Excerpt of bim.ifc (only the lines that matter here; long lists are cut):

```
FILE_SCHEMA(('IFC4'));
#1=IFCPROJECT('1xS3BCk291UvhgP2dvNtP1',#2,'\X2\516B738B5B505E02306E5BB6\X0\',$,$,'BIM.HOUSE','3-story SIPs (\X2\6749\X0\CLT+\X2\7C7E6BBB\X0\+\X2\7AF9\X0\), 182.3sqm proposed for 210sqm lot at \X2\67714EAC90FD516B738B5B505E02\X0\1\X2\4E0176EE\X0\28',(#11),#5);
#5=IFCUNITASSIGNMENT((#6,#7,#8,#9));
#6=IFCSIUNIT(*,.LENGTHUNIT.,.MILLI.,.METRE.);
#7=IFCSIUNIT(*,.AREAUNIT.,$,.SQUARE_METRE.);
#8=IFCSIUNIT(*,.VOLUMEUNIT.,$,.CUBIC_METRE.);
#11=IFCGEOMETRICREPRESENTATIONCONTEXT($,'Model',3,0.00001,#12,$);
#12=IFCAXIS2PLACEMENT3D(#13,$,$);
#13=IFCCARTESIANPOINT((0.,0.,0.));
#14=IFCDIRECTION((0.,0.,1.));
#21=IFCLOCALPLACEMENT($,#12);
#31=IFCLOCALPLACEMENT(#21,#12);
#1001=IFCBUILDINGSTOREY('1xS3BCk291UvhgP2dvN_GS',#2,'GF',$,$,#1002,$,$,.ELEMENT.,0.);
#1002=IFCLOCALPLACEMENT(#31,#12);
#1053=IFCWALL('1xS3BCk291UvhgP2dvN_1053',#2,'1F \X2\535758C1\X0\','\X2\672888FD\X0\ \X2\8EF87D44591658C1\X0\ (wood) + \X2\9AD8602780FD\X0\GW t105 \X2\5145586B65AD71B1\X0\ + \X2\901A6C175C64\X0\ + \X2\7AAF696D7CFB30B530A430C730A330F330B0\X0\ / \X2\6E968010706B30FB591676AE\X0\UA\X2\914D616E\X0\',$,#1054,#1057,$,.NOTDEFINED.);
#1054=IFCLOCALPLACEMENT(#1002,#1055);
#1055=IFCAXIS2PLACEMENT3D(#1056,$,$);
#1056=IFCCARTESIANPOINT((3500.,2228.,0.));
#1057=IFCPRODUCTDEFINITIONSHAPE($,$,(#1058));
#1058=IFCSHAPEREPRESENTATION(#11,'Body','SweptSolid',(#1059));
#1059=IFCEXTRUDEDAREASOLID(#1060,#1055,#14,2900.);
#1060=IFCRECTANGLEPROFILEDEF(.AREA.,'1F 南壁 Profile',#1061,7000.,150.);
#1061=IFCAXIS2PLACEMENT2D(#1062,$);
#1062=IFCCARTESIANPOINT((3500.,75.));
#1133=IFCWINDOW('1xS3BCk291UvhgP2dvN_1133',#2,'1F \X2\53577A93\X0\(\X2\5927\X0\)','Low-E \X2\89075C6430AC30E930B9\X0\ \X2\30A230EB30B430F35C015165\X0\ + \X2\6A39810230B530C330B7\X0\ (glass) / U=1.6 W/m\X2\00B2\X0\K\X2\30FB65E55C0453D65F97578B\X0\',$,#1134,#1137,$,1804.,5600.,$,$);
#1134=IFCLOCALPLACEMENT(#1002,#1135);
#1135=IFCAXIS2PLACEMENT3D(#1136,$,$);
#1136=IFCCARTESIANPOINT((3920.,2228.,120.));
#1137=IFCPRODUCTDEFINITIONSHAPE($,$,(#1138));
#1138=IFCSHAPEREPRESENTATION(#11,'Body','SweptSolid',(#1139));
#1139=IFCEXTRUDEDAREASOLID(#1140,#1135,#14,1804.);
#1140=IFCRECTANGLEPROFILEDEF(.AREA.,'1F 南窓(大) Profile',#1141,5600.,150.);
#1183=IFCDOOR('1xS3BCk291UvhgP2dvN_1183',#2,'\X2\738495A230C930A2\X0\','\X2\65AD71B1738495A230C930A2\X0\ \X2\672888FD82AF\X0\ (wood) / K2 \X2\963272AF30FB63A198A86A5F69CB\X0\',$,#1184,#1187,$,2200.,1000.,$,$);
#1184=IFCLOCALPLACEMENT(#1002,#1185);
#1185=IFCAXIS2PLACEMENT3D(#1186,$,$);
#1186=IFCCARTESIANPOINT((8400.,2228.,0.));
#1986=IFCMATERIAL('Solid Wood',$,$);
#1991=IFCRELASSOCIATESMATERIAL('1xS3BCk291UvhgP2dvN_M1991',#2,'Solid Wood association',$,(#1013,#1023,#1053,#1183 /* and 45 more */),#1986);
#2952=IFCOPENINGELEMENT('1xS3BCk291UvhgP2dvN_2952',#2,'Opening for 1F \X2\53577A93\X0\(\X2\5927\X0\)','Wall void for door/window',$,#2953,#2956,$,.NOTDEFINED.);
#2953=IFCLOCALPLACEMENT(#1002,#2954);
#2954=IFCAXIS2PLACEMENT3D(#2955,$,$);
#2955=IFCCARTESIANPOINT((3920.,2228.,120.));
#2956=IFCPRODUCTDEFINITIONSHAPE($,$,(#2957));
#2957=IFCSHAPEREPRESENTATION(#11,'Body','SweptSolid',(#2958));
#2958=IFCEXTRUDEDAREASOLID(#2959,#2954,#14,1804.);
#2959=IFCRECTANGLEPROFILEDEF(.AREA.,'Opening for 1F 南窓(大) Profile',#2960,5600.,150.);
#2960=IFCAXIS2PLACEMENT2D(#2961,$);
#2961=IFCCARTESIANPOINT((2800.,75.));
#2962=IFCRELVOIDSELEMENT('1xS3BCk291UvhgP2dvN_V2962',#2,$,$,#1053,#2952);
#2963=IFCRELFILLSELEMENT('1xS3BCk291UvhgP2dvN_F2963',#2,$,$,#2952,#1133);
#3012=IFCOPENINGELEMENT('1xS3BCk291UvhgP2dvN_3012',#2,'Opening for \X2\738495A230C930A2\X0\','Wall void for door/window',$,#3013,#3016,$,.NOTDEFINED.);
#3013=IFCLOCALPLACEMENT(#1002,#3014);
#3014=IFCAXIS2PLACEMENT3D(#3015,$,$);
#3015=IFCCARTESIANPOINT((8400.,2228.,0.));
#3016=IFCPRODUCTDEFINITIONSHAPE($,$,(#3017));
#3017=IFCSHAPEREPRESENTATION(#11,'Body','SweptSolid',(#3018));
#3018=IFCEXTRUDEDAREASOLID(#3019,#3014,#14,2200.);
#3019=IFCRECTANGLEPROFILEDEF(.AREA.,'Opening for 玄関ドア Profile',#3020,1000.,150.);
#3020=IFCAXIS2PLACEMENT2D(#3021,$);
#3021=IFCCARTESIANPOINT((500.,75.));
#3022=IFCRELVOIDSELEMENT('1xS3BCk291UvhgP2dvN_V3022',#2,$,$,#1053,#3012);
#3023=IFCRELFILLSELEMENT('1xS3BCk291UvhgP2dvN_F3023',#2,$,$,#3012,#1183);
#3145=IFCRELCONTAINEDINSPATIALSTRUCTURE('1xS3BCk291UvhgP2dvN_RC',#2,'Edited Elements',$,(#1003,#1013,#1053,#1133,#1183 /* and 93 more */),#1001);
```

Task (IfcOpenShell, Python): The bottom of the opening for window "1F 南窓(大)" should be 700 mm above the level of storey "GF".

```python
import numpy as np
import ifcopenshell
import ifcopenshell.api.geometry
import ifcopenshell.geom
import ifcopenshell.util.element
import ifcopenshell.util.placement
import ifcopenshell.util.shape
import ifcopenshell.util.unit

model = ifcopenshell.open("bim.ifc")
unit_scale = ifcopenshell.util.unit.calculate_unit_scale(model)

window = model.by_id(1133)
opening = window.FillsVoids[0].RelatingOpeningElement
storey = ifcopenshell.util.element.get_container(window, ifc_class="IfcBuildingStorey")
level = ifcopenshell.util.placement.get_local_placement(storey.ObjectPlacement)[2, 3]

# The opening's origin need not be at the sill, so measure its lowest point.
shape = ifcopenshell.geom.create_shape(ifcopenshell.geom.settings(), opening)
bottom = ifcopenshell.util.shape.get_shape_bottom_elevation(shape, shape.geometry) / unit_scale
dz = level + 700.0 - bottom

shift = np.array([0.0, 0.0, dz])
# The window is not placed relative to its opening, so move both.
for product in (opening, window):
    matrix = ifcopenshell.util.placement.get_local_placement(product.ObjectPlacement)
    matrix[:3, 3] += shift
    ifcopenshell.api.geometry.edit_object_placement(model, product=product, matrix=matrix, is_si=False)

print(f"moved by {dz * unit_scale:+.3f} m")

model.write("bim_updated.ifc")
```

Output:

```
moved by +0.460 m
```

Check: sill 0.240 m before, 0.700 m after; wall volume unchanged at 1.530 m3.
